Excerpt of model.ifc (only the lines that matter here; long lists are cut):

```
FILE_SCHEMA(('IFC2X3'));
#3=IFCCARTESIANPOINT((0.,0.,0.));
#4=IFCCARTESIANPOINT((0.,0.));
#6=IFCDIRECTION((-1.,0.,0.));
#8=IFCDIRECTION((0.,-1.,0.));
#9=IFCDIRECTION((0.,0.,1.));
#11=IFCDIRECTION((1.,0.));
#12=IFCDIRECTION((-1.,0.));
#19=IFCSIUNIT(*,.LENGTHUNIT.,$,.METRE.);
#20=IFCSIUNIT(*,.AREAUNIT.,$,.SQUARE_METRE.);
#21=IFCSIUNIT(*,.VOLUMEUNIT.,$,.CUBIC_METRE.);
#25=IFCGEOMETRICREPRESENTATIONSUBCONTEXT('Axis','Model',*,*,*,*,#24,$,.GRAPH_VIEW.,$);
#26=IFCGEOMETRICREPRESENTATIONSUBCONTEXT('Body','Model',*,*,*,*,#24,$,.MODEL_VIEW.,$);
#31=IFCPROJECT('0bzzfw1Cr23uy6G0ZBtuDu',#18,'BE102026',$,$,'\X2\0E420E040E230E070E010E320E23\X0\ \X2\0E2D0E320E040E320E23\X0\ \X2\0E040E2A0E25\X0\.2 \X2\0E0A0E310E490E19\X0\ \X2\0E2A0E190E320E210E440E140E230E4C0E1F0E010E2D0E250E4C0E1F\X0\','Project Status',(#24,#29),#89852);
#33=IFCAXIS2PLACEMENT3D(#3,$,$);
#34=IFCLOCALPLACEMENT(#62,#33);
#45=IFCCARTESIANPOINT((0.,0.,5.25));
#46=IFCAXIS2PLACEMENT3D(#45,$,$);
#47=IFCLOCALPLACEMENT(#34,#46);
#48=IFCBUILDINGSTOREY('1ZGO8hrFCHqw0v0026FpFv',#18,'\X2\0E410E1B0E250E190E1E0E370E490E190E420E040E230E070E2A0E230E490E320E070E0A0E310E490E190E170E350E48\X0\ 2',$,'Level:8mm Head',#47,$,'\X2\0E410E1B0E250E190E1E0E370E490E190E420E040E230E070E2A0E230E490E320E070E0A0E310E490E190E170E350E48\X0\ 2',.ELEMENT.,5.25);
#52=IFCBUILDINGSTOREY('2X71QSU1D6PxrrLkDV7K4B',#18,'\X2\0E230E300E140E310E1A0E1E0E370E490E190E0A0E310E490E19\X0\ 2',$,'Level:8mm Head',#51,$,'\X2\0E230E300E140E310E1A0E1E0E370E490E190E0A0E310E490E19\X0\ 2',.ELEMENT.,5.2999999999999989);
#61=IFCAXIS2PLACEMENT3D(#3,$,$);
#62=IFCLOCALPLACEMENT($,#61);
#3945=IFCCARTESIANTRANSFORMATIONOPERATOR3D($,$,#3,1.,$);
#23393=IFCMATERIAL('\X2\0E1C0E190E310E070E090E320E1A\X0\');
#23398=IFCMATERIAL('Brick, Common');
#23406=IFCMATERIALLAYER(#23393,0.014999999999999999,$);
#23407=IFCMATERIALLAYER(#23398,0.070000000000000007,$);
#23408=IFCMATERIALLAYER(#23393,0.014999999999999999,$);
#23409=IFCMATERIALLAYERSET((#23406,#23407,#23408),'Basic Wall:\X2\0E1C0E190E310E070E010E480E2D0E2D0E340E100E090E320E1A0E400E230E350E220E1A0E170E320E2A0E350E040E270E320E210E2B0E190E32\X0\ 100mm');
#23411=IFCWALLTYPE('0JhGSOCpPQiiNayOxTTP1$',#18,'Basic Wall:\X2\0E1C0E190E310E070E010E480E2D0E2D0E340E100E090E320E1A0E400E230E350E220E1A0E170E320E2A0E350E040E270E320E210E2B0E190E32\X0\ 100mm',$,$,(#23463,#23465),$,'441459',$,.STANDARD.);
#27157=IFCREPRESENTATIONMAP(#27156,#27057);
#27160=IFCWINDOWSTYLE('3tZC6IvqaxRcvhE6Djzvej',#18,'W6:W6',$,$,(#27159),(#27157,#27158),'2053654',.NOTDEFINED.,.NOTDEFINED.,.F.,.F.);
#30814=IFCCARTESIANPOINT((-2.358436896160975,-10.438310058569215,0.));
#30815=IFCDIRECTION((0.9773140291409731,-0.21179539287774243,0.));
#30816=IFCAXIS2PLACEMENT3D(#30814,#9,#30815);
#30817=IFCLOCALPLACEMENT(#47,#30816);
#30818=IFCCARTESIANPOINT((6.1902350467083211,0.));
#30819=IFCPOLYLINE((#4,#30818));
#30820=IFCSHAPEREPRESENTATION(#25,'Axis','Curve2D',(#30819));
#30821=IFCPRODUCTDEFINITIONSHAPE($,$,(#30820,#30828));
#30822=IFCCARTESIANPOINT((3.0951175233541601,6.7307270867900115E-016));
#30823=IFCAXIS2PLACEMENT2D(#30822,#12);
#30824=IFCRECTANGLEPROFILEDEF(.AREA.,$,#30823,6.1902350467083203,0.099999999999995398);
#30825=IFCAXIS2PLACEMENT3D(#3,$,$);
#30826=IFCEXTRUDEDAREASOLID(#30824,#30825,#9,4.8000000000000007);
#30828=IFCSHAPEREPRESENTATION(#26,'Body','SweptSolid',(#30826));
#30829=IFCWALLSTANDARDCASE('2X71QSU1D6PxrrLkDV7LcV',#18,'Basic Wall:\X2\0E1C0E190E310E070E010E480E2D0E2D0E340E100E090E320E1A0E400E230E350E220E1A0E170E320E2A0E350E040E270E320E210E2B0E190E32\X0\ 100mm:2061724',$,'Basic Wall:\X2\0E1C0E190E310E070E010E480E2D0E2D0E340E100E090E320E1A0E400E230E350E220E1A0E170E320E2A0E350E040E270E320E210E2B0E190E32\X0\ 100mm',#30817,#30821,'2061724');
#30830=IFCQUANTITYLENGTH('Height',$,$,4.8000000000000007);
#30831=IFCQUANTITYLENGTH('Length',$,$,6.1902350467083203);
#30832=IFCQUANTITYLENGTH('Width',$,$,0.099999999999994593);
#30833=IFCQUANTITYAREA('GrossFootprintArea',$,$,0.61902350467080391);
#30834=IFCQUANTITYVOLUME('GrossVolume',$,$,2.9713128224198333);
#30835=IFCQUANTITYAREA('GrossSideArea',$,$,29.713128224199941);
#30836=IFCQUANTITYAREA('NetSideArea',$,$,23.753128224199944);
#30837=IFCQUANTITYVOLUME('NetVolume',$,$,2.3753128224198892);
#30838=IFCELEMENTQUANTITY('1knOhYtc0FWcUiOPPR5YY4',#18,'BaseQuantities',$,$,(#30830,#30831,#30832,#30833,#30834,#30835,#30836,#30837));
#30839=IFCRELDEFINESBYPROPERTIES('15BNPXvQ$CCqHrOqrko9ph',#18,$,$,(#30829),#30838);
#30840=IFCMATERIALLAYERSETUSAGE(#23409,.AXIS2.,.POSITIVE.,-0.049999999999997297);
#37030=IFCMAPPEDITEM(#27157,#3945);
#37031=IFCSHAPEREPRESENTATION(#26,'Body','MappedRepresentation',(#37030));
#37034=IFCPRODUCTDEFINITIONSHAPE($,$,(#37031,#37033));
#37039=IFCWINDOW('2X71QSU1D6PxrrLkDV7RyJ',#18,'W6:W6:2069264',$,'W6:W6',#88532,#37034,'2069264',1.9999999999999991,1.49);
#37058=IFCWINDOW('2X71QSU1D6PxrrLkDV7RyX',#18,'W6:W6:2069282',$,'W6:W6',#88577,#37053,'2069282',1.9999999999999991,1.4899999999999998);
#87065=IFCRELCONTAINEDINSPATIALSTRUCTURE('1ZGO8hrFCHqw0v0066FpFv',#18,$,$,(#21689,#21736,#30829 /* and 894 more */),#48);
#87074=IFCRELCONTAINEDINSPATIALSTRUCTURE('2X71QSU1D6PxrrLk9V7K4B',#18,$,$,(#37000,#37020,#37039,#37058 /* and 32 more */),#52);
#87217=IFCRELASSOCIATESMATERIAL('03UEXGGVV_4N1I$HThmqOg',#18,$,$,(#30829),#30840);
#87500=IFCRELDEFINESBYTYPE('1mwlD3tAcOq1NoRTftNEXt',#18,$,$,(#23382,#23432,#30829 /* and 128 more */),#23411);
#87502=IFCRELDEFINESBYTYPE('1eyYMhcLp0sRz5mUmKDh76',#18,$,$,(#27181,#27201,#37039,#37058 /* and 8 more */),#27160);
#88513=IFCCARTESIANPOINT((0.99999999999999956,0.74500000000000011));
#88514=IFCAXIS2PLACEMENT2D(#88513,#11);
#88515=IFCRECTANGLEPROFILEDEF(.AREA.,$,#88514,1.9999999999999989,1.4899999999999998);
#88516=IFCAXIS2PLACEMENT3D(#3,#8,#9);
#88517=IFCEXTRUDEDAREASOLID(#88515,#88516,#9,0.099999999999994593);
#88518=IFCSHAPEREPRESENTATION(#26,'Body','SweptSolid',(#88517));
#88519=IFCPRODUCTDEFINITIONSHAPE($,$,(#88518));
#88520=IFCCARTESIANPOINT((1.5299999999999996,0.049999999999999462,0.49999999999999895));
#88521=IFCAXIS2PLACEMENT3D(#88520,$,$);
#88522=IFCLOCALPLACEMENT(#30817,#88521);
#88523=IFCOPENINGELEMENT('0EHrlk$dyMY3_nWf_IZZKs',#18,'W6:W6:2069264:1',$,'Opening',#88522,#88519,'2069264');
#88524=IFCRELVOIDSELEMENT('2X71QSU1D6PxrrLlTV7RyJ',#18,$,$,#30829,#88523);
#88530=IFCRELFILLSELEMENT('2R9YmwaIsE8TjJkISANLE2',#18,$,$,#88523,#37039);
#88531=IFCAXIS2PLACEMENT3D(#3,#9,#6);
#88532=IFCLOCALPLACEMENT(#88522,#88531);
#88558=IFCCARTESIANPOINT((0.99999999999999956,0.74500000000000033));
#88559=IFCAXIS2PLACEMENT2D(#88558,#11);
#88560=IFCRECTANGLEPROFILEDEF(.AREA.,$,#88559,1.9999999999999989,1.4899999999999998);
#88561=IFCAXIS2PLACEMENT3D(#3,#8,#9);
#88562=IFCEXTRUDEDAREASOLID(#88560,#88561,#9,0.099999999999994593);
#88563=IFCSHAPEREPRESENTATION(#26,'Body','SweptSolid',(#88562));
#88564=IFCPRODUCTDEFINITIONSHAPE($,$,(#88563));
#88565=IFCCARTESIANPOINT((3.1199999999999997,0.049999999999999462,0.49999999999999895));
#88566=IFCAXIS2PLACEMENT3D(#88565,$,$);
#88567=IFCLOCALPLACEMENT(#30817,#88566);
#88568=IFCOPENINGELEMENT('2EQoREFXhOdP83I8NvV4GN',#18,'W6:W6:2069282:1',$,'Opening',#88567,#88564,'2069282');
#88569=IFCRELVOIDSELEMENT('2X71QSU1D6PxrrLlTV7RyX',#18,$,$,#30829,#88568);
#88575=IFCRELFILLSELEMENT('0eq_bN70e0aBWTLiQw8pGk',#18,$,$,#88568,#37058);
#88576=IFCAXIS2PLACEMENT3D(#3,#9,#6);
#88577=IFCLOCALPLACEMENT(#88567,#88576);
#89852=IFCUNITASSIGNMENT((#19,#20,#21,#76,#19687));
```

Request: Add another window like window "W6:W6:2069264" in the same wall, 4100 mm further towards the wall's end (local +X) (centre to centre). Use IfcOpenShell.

```python
import ifcopenshell
import ifcopenshell.api.feature
import ifcopenshell.api.geometry
import ifcopenshell.api.pset
import ifcopenshell.api.root
import ifcopenshell.geom
import ifcopenshell.util.element
import ifcopenshell.util.placement
import ifcopenshell.util.shape
import ifcopenshell.util.unit

model = ifcopenshell.open("model.ifc")
unit_scale = ifcopenshell.util.unit.calculate_unit_scale(model)
area_scale = ifcopenshell.util.unit.calculate_unit_scale(model, "AREAUNIT")
volume_scale = ifcopenshell.util.unit.calculate_unit_scale(model, "VOLUMEUNIT")
settings = ifcopenshell.geom.settings()


def volume(element):
    """Net volume in cubic metres, openings subtracted."""
    shape = ifcopenshell.geom.create_shape(settings, element)
    return ifcopenshell.util.shape.get_volume(shape.geometry)


def reuse_history(source, copy):
    """copy_class also copies each property set's owner history, people and application; keep the originals."""
    for rel in copy.IsDefinedBy:
        if rel.is_a("IfcRelDefinesByProperties") and (history := rel.RelatingPropertyDefinition.OwnerHistory):
            rel.RelatingPropertyDefinition.OwnerHistory = source.OwnerHistory
            ifcopenshell.util.element.remove_deep2(model, history)


window = model.by_guid("2X71QSU1D6PxrrLkDV7RyJ")
opening = window.FillsVoids[0].RelatingOpeningElement
wall = opening.VoidsElements[0].RelatingBuildingElement
before = volume(wall)
shift = ifcopenshell.util.placement.get_local_placement(wall.ObjectPlacement)[:3, 0] * 4.1 / unit_scale

# copy_class copies the void relationship, type, container and properties, but no geometry.
new_opening = ifcopenshell.api.root.copy_class(model, product=opening)
new_opening.Representation = ifcopenshell.util.element.copy_deep(
    model, opening.Representation, exclude=["IfcGeometricRepresentationContext", "IfcRepresentationMap"]
)
new_opening.Name = "W6:W6"
new_opening.Tag = None
reuse_history(opening, new_opening)
new_window = ifcopenshell.api.root.copy_class(model, product=window)
new_window.Representation = ifcopenshell.util.element.copy_deep(
    model, window.Representation, exclude=["IfcGeometricRepresentationContext", "IfcRepresentationMap"]
)
new_window.Name = "W6:W6"
new_window.Tag = None
reuse_history(window, new_window)
fills = ifcopenshell.api.feature.add_filling(model, opening=new_opening, element=new_window)
fills.OwnerHistory = new_window.OwnerHistory  # required in IFC2X3

for old, new in ((opening, new_opening), (window, new_window)):
    matrix = ifcopenshell.util.placement.get_local_placement(old.ObjectPlacement)
    matrix[:3, 3] += shift
    ifcopenshell.api.geometry.edit_object_placement(model, product=new, matrix=matrix, is_si=False)

after = volume(wall)
thickness = 0.1  # wall thickness in metres

# Update the wall's stored quantities.
qto = model.by_id(ifcopenshell.util.element.get_pset(wall, "BaseQuantities", should_inherit=False)["id"])
ifcopenshell.api.pset.edit_qto(model, qto=qto, properties={
    "NetSideArea": after / thickness / area_scale,
    "NetVolume": after / volume_scale,
})

print(f"wall volume {before:.3f} -> {after:.3f} m3")

model.write("model-out.ifc")
```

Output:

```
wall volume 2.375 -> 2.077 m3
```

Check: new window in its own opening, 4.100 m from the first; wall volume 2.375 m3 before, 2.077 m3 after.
